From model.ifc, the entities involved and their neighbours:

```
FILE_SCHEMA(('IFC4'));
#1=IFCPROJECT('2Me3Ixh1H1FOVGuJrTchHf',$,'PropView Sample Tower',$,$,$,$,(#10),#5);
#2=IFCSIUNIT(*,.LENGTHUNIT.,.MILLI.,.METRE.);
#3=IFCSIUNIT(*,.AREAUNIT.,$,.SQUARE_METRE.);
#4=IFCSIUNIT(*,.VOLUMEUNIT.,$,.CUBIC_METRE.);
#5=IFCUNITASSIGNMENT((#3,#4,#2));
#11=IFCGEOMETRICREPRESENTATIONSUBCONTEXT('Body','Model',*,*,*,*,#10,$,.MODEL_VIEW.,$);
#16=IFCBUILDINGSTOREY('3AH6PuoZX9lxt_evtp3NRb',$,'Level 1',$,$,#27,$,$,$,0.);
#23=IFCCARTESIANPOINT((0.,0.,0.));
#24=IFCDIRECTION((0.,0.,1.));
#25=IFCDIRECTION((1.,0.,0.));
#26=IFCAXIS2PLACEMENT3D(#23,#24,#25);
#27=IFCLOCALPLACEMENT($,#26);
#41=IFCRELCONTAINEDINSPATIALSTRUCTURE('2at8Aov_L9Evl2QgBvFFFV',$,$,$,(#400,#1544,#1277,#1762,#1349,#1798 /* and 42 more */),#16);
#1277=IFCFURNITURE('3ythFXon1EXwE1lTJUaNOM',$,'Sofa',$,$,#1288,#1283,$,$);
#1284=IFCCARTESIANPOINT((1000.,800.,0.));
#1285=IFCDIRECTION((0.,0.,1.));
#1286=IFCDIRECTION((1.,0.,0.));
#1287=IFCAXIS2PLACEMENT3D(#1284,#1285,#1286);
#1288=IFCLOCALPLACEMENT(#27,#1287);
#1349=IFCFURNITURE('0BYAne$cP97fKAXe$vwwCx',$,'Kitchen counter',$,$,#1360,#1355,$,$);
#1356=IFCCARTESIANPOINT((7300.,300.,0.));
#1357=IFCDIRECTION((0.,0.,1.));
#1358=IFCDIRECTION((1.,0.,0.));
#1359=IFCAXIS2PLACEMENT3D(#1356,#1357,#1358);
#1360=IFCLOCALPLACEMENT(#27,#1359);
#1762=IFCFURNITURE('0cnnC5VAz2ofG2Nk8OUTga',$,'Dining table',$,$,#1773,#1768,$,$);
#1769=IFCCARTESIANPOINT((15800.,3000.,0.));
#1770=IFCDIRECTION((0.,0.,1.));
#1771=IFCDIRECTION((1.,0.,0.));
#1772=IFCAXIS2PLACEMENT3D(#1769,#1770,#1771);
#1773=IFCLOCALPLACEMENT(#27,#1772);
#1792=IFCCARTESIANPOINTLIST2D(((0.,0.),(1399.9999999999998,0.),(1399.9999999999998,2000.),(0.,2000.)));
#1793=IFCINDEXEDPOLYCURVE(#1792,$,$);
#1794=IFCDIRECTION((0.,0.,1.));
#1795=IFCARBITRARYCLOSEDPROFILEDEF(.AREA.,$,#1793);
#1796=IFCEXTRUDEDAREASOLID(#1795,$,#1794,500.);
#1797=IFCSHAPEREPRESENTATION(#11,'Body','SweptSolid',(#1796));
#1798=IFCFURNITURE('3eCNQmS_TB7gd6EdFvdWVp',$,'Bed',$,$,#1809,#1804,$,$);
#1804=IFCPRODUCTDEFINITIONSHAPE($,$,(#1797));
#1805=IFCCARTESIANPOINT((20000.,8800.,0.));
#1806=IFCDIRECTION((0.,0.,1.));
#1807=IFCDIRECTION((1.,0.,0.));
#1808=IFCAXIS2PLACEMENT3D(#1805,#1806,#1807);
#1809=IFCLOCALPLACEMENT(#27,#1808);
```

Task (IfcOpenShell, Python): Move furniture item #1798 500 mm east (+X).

```python
import ifcopenshell
import ifcopenshell.api.geometry
import ifcopenshell.util.placement
import ifcopenshell.util.unit

model = ifcopenshell.open("model.ifc")
unit_scale = ifcopenshell.util.unit.calculate_unit_scale(model)

item = model.by_guid("3eCNQmS_TB7gd6EdFvdWVp")
matrix = ifcopenshell.util.placement.get_local_placement(item.ObjectPlacement)
matrix[0, 3] += 0.5 / unit_scale
ifcopenshell.api.geometry.edit_object_placement(model, product=item, matrix=matrix, is_si=False)

print(ifcopenshell.util.placement.get_local_placement(item.ObjectPlacement).round(3) + 0.0)

model.write("model-out.ifc")
```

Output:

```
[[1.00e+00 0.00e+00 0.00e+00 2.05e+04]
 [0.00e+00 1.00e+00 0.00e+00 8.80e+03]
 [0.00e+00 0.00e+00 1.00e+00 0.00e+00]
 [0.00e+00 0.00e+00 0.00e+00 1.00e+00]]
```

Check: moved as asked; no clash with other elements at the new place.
